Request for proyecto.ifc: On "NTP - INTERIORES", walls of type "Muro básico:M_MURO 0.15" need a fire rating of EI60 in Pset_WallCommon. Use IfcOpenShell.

First a look at what the model holds.

```python
import ifcopenshell
import ifcopenshell.util.element

model = ifcopenshell.open("proyecto.ifc")
print(model.schema)
storey = next(s for s in model.by_type("IfcBuildingStorey") if s.Name == "NTP - INTERIORES")
walls = [e for e in ifcopenshell.util.element.get_decomposition(storey) if e.is_a("IfcWall")]
seen = {}
for e in walls:
    element_type = ifcopenshell.util.element.get_type(e)
    key = (element_type.Name if element_type != e and element_type else None, ifcopenshell.util.element.get_pset(e, "Pset_WallCommon", "FireRating"))
    seen[key] = seen.get(key, 0) + 1
for (name, value), count in sorted(seen.items(), key=str):
    print(count, "x", name, "|", value)
```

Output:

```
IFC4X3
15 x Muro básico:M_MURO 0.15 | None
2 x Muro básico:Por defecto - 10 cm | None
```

```python
import ifcopenshell
import ifcopenshell.api.pset
import ifcopenshell.util.element

model = ifcopenshell.open("proyecto.ifc")

storey = next(s for s in model.by_type("IfcBuildingStorey") if s.Name == "NTP - INTERIORES")
walls = [e for e in ifcopenshell.util.element.get_decomposition(storey) if e.is_a("IfcWall")]

count = 0
for e in walls:
    element_type = ifcopenshell.util.element.get_type(e)
    if element_type in (None, e) or element_type.Name != "Muro básico:M_MURO 0.15":
        continue
    # add_pset returns the element's existing set when there is one.
    pset = ifcopenshell.api.pset.add_pset(model, product=e, name="Pset_WallCommon")
    ifcopenshell.api.pset.edit_pset(model, pset=pset, properties={"FireRating": "EI60"})
    count += 1

print(count, "walls updated")

model.write("proyecto_rev.ifc")
```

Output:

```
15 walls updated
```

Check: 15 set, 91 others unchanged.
